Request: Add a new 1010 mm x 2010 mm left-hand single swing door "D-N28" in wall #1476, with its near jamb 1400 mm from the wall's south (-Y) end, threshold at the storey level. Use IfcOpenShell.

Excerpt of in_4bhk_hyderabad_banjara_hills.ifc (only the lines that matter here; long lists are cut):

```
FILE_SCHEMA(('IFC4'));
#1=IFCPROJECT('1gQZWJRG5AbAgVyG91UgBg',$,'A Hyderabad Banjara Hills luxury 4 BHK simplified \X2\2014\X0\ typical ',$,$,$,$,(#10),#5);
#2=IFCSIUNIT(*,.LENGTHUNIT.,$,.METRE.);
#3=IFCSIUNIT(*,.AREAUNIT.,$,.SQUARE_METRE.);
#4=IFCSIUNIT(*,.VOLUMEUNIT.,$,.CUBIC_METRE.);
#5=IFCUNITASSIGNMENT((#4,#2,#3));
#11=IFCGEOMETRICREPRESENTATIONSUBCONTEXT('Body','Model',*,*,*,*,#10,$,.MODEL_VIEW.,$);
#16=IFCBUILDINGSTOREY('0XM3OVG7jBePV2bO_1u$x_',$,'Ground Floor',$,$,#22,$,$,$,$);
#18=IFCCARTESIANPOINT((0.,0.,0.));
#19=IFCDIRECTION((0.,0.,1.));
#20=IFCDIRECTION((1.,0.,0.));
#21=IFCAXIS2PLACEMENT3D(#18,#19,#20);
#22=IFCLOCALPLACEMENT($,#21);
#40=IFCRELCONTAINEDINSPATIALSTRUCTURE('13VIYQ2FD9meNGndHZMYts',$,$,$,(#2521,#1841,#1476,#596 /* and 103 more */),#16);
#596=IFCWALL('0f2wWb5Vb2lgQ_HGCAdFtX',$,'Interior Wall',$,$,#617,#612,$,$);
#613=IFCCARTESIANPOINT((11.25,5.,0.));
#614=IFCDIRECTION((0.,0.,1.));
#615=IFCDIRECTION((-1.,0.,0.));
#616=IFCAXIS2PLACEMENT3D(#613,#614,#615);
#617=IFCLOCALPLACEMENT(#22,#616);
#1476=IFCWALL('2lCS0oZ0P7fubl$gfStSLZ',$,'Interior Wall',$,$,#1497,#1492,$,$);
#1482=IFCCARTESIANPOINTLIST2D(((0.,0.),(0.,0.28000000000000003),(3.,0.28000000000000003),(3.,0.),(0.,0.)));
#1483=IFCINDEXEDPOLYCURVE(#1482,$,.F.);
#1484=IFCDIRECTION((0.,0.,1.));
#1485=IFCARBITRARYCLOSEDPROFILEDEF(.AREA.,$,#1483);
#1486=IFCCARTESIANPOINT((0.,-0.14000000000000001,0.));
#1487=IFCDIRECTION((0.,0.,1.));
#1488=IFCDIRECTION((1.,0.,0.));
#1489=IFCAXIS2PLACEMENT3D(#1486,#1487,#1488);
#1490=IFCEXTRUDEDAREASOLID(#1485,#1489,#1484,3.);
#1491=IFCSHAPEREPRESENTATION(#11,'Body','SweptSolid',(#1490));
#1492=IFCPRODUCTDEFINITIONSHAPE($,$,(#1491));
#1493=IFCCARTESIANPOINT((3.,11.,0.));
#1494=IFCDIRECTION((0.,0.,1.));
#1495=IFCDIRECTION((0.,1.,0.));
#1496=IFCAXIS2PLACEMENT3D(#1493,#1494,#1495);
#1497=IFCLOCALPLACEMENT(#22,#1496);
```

```python
import numpy as np
import ifcopenshell
import ifcopenshell.api.feature
import ifcopenshell.api.geometry
import ifcopenshell.api.root
import ifcopenshell.api.spatial
import ifcopenshell.geom
import ifcopenshell.util.element
import ifcopenshell.util.placement
import ifcopenshell.util.representation
import ifcopenshell.util.shape
import ifcopenshell.util.unit

model = ifcopenshell.open("in_4bhk_hyderabad_banjara_hills.ifc")
unit_scale = ifcopenshell.util.unit.calculate_unit_scale(model)
settings = ifcopenshell.geom.settings()


def volume(element):
    """Net volume in cubic metres, openings subtracted."""
    shape = ifcopenshell.geom.create_shape(settings, element)
    return ifcopenshell.util.shape.get_volume(shape.geometry)


wall = model.by_guid("2lCS0oZ0P7fubl$gfStSLZ")
storey = ifcopenshell.util.element.get_container(wall, ifc_class="IfcBuildingStorey")
context = ifcopenshell.util.representation.get_context(model, "Model", "Body", "MODEL_VIEW")
before = volume(wall)

width, height, from_end, sill = 1.01, 2.01, 1.4, 0.0  # metres

# The wall runs along its own X axis, and the end named is its -X end.
wall_shape = ifcopenshell.geom.create_shape(settings, wall)
x, y, z = ifcopenshell.util.shape.get_vertices(wall_shape.geometry).T
start = x.min() + from_end
face, thickness = float(y.min()), float(y.max() - y.min())
wall_matrix = ifcopenshell.util.placement.get_local_placement(wall.ObjectPlacement)
level = ifcopenshell.util.placement.get_local_placement(storey.ObjectPlacement)[2, 3]


def in_wall(x, y):
    """Placement at x, y metres in the wall's axes, at sill height."""
    matrix = wall_matrix.copy()
    matrix[:, 3] = wall_matrix @ np.array([x / unit_scale, y / unit_scale, 0.0, 1.0])
    matrix[2, 3] = level + sill / unit_scale
    return matrix


# Opening: a box that overshoots both wall faces by 50 mm.
opening = ifcopenshell.api.root.create_entity(model, ifc_class="IfcOpeningElement", predefined_type="OPENING")
box = ifcopenshell.api.geometry.add_wall_representation(
    model, context=context, length=width, height=height, thickness=thickness + 0.1
)
ifcopenshell.api.geometry.assign_representation(model, product=opening, representation=box)
ifcopenshell.api.geometry.edit_object_placement(model, product=opening, matrix=in_wall(start, face - 0.05), is_si=False)
ifcopenshell.api.feature.add_feature(model, feature=opening, element=wall)

door = ifcopenshell.api.root.create_entity(model, ifc_class="IfcDoor", name="D-N28", predefined_type="DOOR")
door.OverallWidth, door.OverallHeight = width / unit_scale, height / unit_scale
door.OperationType = "SINGLE_SWING_LEFT"
body = ifcopenshell.api.geometry.add_door_representation(
    model,
    context=context,
    overall_width=door.OverallWidth,
    overall_height=door.OverallHeight,
    operation_type="SINGLE_SWING_LEFT",
    lining_properties={"LiningDepth": thickness / unit_scale, "ThresholdDepth": thickness / unit_scale},
)
ifcopenshell.api.geometry.assign_representation(model, product=door, representation=body)
ifcopenshell.api.spatial.assign_container(model, products=[door], relating_structure=storey)
ifcopenshell.api.feature.add_filling(model, opening=opening, element=door)

# The lining spans the wall, so the door starts at the wall face.
ifcopenshell.api.geometry.edit_object_placement(model, product=door, matrix=in_wall(start, face), is_si=False)

after = volume(wall)

print(f"wall volume {before:.3f} -> {after:.3f} m3")

model.write("in_4bhk_hyderabad_banjara_hills_updated.ifc")
```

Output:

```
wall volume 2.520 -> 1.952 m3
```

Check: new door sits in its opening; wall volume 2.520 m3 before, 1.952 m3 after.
